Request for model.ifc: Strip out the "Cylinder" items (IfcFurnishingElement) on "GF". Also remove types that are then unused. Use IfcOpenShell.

First a look at what the model holds.

```python
import ifcopenshell
import ifcopenshell.util.element

model = ifcopenshell.open("model.ifc")
print(model.schema)
storey = next(s for s in model.by_type("IfcBuildingStorey") if s.Name == "GF")
furniture = [e for e in ifcopenshell.util.element.get_decomposition(storey) if e.is_a("IfcFurnishingElement")]
seen = {}
for e in furniture:
    element_type = ifcopenshell.util.element.get_type(e)
    name = element_type.Name if element_type not in (None, e) else None
    seen[name] = seen.get(name, 0) + 1
for name, count in sorted(seen.items(), key=str):
    print(count, "x", name)
```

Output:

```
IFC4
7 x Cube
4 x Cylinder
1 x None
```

```python
import ifcopenshell
import ifcopenshell.api.root
import ifcopenshell.util.element

model = ifcopenshell.open("model.ifc")

storey = next(s for s in model.by_type("IfcBuildingStorey") if s.Name == "GF")
furniture = [e for e in ifcopenshell.util.element.get_decomposition(storey) if e.is_a("IfcFurnishingElement")]
targets = [e for e in furniture if (t := ifcopenshell.util.element.get_type(e)) not in (None, e) and t.Name == "Cylinder"]
types = {ifcopenshell.util.element.get_type(e) for e in targets} - {None, *targets}

for e in targets:
    ifcopenshell.api.root.remove_product(model, product=e)
print(len(targets), "removed")

unused = [t for t in types if not ifcopenshell.util.element.get_types(t)]
for t in unused:
    ifcopenshell.api.root.remove_product(model, product=t)
print(len(unused), "unused types removed")

model.write("model_rev.ifc")
```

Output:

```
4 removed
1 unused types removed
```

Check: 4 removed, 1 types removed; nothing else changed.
